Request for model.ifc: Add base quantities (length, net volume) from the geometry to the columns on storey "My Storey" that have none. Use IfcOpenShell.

First a look at what the model holds.

```python
import ifcopenshell
import ifcopenshell.util.element
import ifcopenshell.util.unit

model = ifcopenshell.open("model.ifc")
print(model.schema)
for unit_type in ("LENGTHUNIT", "AREAUNIT", "VOLUMEUNIT"):
    print(unit_type, ifcopenshell.util.unit.calculate_unit_scale(model, unit_type))
storey = next(s for s in model.by_type("IfcBuildingStorey") if s.Name == "My Storey")
columns = [e for e in ifcopenshell.util.element.get_decomposition(storey) if e.is_a("IfcColumn")]
for e in sorted(columns, key=lambda e: e.id()):
    print(e.id(), e.is_a(), e.Name, list(ifcopenshell.util.element.get_psets(e, qtos_only=True)), sep=" | ")
```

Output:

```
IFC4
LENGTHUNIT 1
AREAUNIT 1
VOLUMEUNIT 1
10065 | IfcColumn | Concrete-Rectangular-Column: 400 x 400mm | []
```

```python
import ifcopenshell
import ifcopenshell.api.pset
import ifcopenshell.geom
import ifcopenshell.util.element
import ifcopenshell.util.shape
import ifcopenshell.util.unit

model = ifcopenshell.open("model.ifc")
unit_scale = ifcopenshell.util.unit.calculate_unit_scale(model)
volume_scale = ifcopenshell.util.unit.calculate_unit_scale(model, "VOLUMEUNIT")
settings = ifcopenshell.geom.settings()

storey = next(s for s in model.by_type("IfcBuildingStorey") if s.Name == "My Storey")
columns = [e for e in ifcopenshell.util.element.get_decomposition(storey) if e.is_a("IfcColumn")]

for e in sorted(columns, key=lambda e: e.id()):
    if ifcopenshell.util.element.get_psets(e, qtos_only=True, should_inherit=False):
        continue
    # Geometry comes back in metres, in the element's own axes.
    shape = ifcopenshell.geom.create_shape(settings, e)
    values = {
        "Length": ifcopenshell.util.shape.get_z(shape.geometry) / unit_scale,
        "NetVolume": ifcopenshell.util.shape.get_volume(shape.geometry) / volume_scale,
    }
    qto = ifcopenshell.api.pset.add_qto(model, product=e, name="Qto_ColumnBaseQuantities")
    ifcopenshell.api.pset.edit_qto(model, qto=qto, properties=values)
    print(e.id(), {k: round(v, 3) for k, v in values.items()})

model.write("model_edited.ifc")
```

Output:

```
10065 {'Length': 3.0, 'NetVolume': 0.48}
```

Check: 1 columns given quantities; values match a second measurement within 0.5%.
